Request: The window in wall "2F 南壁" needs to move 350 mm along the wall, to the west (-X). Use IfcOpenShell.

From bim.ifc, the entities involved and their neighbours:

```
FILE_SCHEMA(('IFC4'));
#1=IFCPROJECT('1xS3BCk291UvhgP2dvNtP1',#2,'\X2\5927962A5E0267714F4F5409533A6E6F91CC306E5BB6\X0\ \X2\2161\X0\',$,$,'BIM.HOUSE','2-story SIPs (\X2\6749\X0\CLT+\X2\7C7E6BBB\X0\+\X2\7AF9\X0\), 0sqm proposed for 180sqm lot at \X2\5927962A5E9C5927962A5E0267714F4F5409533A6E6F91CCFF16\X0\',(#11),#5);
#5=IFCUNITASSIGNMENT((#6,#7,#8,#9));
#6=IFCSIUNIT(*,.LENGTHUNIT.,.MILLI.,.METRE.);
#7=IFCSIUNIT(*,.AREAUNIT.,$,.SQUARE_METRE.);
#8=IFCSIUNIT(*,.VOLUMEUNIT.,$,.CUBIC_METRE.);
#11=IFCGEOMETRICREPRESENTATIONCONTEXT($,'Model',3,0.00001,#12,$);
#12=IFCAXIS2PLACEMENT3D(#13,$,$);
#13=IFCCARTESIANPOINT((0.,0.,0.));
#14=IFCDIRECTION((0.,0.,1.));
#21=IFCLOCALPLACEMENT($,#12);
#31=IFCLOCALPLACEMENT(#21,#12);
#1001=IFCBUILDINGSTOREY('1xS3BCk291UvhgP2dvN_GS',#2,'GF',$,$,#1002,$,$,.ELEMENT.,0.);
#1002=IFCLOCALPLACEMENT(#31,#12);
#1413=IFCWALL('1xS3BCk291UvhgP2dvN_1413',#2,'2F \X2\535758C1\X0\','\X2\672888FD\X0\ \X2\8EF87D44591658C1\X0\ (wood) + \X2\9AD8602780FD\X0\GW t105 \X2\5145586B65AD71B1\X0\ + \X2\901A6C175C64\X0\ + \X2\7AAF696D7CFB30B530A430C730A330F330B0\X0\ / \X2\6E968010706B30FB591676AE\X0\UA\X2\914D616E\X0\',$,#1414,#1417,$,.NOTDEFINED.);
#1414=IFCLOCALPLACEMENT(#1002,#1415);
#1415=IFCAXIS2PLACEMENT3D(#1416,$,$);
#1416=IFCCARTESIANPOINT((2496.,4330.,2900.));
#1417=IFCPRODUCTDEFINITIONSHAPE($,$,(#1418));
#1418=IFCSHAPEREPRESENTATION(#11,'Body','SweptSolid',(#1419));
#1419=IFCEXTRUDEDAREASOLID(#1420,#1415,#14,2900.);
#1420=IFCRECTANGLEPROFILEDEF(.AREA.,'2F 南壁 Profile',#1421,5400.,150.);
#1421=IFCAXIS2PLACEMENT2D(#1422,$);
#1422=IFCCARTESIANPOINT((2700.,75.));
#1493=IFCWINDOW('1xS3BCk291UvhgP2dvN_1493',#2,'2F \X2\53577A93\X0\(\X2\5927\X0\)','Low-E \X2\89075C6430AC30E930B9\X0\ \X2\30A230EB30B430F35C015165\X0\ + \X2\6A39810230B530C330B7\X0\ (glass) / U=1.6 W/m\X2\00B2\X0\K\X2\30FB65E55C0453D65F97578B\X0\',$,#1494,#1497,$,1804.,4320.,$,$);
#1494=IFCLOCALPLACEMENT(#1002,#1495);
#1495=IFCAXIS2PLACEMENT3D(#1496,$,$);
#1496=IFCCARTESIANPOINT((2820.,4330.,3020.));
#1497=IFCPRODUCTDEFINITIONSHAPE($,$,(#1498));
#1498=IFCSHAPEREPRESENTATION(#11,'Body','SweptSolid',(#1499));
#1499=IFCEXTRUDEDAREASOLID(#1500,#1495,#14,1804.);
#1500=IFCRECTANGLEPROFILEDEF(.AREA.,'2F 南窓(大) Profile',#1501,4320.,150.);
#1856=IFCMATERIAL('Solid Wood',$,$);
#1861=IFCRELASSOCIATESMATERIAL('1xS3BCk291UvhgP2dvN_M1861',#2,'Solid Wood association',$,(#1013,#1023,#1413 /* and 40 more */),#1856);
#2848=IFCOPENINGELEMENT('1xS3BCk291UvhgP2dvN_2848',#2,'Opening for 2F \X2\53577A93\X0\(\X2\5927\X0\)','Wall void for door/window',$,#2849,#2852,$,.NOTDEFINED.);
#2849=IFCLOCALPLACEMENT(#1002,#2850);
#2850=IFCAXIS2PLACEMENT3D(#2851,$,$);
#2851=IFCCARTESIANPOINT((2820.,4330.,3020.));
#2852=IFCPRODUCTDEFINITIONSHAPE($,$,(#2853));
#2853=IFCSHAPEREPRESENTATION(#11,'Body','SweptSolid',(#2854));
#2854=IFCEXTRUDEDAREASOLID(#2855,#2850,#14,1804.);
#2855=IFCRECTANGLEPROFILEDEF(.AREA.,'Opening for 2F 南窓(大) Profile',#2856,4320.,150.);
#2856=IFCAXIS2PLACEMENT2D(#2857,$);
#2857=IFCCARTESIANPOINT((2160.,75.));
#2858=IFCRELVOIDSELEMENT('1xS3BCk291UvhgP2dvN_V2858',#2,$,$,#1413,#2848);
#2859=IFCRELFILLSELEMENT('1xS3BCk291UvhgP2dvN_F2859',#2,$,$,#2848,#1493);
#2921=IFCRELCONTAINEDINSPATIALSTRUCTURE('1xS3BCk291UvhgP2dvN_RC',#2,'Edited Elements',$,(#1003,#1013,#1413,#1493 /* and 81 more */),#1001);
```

```python
import ifcopenshell
import ifcopenshell.api.geometry
import ifcopenshell.util.placement
import ifcopenshell.util.unit

model = ifcopenshell.open("bim.ifc")
unit_scale = ifcopenshell.util.unit.calculate_unit_scale(model)

window = model.by_guid("1xS3BCk291UvhgP2dvN_1493")
opening = window.FillsVoids[0].RelatingOpeningElement
wall = opening.VoidsElements[0].RelatingBuildingElement

wall_matrix = ifcopenshell.util.placement.get_local_placement(wall.ObjectPlacement)
shift = wall_matrix[:3, 0] * -0.35 / unit_scale
before = ifcopenshell.util.placement.get_local_placement(window.ObjectPlacement)[:3, 3].copy()

# The window is not placed relative to its opening, so move both.
for product in (opening, window):
    matrix = ifcopenshell.util.placement.get_local_placement(product.ObjectPlacement)
    matrix[:3, 3] += shift
    ifcopenshell.api.geometry.edit_object_placement(model, product=product, matrix=matrix, is_si=False)

after = ifcopenshell.util.placement.get_local_placement(window.ObjectPlacement)[:3, 3]
print("window moved by", (after - before).round(3) + 0.0)

model.write("bim_v2.ifc")
```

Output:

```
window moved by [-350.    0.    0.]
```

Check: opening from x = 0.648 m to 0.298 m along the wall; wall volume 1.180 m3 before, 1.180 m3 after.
